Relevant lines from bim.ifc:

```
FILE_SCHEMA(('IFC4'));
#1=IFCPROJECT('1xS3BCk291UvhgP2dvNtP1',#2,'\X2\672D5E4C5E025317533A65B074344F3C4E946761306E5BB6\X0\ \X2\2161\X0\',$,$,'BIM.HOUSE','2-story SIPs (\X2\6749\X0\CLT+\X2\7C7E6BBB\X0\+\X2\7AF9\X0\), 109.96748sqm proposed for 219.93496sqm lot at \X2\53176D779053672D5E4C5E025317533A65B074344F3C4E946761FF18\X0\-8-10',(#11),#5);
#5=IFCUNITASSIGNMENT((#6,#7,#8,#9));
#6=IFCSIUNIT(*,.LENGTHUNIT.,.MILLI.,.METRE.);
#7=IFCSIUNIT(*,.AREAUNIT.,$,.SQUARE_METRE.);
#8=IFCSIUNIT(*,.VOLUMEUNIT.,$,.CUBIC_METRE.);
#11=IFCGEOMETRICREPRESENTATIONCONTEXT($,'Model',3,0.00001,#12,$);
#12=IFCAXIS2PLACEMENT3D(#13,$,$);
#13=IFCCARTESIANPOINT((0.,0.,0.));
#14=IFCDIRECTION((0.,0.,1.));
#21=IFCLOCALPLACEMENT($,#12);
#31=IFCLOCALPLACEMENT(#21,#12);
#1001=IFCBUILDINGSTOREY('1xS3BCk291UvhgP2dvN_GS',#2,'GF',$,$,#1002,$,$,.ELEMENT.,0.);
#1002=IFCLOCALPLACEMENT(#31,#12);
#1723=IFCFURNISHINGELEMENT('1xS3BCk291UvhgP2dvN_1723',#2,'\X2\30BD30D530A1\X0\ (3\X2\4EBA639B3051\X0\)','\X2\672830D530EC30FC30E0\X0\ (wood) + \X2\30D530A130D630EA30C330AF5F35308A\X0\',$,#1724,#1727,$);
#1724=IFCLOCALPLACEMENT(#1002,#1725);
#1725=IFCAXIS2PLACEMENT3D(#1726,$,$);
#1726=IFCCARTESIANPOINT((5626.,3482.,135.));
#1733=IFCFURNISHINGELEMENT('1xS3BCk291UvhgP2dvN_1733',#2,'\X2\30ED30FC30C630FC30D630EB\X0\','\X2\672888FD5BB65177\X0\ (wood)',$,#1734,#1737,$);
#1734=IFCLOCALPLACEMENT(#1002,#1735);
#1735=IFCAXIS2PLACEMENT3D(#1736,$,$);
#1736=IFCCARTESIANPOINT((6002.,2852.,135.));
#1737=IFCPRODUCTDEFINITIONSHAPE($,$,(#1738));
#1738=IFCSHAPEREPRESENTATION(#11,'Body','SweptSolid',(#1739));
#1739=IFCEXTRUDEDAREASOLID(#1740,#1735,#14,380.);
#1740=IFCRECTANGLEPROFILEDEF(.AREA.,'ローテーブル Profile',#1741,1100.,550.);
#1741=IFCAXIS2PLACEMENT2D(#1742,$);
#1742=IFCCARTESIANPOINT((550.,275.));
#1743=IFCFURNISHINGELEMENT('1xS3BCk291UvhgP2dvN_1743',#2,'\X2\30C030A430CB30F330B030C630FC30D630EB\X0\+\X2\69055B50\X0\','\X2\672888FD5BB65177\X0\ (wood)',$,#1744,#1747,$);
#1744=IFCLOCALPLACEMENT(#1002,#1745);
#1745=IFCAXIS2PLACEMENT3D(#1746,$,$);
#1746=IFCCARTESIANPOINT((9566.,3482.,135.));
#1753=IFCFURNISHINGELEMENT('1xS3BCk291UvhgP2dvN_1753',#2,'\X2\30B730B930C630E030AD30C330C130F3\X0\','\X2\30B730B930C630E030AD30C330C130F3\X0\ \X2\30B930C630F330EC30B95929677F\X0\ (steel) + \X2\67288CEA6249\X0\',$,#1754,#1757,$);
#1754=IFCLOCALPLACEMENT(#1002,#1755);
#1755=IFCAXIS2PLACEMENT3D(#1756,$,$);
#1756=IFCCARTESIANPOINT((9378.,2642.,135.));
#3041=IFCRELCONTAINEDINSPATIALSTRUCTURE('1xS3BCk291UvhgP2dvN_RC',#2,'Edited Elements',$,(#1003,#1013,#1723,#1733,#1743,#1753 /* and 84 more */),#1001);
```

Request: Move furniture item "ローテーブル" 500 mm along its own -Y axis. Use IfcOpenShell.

```python
import ifcopenshell
import ifcopenshell.api.geometry
import ifcopenshell.util.placement

model = ifcopenshell.open("bim.ifc")

item = model.by_guid("1xS3BCk291UvhgP2dvN_1733")
matrix = ifcopenshell.util.placement.get_local_placement(item.ObjectPlacement)
matrix[:3, 3] -= matrix[:3, 1] * 500.0
ifcopenshell.api.geometry.edit_object_placement(model, product=item, matrix=matrix, is_si=False)

print(ifcopenshell.util.placement.get_local_placement(item.ObjectPlacement).round(3) + 0.0)

model.write("bim_edited.ifc")
```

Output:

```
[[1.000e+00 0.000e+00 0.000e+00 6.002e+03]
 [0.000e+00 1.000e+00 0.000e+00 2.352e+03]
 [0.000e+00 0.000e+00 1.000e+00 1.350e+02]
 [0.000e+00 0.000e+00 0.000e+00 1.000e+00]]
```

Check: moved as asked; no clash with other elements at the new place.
